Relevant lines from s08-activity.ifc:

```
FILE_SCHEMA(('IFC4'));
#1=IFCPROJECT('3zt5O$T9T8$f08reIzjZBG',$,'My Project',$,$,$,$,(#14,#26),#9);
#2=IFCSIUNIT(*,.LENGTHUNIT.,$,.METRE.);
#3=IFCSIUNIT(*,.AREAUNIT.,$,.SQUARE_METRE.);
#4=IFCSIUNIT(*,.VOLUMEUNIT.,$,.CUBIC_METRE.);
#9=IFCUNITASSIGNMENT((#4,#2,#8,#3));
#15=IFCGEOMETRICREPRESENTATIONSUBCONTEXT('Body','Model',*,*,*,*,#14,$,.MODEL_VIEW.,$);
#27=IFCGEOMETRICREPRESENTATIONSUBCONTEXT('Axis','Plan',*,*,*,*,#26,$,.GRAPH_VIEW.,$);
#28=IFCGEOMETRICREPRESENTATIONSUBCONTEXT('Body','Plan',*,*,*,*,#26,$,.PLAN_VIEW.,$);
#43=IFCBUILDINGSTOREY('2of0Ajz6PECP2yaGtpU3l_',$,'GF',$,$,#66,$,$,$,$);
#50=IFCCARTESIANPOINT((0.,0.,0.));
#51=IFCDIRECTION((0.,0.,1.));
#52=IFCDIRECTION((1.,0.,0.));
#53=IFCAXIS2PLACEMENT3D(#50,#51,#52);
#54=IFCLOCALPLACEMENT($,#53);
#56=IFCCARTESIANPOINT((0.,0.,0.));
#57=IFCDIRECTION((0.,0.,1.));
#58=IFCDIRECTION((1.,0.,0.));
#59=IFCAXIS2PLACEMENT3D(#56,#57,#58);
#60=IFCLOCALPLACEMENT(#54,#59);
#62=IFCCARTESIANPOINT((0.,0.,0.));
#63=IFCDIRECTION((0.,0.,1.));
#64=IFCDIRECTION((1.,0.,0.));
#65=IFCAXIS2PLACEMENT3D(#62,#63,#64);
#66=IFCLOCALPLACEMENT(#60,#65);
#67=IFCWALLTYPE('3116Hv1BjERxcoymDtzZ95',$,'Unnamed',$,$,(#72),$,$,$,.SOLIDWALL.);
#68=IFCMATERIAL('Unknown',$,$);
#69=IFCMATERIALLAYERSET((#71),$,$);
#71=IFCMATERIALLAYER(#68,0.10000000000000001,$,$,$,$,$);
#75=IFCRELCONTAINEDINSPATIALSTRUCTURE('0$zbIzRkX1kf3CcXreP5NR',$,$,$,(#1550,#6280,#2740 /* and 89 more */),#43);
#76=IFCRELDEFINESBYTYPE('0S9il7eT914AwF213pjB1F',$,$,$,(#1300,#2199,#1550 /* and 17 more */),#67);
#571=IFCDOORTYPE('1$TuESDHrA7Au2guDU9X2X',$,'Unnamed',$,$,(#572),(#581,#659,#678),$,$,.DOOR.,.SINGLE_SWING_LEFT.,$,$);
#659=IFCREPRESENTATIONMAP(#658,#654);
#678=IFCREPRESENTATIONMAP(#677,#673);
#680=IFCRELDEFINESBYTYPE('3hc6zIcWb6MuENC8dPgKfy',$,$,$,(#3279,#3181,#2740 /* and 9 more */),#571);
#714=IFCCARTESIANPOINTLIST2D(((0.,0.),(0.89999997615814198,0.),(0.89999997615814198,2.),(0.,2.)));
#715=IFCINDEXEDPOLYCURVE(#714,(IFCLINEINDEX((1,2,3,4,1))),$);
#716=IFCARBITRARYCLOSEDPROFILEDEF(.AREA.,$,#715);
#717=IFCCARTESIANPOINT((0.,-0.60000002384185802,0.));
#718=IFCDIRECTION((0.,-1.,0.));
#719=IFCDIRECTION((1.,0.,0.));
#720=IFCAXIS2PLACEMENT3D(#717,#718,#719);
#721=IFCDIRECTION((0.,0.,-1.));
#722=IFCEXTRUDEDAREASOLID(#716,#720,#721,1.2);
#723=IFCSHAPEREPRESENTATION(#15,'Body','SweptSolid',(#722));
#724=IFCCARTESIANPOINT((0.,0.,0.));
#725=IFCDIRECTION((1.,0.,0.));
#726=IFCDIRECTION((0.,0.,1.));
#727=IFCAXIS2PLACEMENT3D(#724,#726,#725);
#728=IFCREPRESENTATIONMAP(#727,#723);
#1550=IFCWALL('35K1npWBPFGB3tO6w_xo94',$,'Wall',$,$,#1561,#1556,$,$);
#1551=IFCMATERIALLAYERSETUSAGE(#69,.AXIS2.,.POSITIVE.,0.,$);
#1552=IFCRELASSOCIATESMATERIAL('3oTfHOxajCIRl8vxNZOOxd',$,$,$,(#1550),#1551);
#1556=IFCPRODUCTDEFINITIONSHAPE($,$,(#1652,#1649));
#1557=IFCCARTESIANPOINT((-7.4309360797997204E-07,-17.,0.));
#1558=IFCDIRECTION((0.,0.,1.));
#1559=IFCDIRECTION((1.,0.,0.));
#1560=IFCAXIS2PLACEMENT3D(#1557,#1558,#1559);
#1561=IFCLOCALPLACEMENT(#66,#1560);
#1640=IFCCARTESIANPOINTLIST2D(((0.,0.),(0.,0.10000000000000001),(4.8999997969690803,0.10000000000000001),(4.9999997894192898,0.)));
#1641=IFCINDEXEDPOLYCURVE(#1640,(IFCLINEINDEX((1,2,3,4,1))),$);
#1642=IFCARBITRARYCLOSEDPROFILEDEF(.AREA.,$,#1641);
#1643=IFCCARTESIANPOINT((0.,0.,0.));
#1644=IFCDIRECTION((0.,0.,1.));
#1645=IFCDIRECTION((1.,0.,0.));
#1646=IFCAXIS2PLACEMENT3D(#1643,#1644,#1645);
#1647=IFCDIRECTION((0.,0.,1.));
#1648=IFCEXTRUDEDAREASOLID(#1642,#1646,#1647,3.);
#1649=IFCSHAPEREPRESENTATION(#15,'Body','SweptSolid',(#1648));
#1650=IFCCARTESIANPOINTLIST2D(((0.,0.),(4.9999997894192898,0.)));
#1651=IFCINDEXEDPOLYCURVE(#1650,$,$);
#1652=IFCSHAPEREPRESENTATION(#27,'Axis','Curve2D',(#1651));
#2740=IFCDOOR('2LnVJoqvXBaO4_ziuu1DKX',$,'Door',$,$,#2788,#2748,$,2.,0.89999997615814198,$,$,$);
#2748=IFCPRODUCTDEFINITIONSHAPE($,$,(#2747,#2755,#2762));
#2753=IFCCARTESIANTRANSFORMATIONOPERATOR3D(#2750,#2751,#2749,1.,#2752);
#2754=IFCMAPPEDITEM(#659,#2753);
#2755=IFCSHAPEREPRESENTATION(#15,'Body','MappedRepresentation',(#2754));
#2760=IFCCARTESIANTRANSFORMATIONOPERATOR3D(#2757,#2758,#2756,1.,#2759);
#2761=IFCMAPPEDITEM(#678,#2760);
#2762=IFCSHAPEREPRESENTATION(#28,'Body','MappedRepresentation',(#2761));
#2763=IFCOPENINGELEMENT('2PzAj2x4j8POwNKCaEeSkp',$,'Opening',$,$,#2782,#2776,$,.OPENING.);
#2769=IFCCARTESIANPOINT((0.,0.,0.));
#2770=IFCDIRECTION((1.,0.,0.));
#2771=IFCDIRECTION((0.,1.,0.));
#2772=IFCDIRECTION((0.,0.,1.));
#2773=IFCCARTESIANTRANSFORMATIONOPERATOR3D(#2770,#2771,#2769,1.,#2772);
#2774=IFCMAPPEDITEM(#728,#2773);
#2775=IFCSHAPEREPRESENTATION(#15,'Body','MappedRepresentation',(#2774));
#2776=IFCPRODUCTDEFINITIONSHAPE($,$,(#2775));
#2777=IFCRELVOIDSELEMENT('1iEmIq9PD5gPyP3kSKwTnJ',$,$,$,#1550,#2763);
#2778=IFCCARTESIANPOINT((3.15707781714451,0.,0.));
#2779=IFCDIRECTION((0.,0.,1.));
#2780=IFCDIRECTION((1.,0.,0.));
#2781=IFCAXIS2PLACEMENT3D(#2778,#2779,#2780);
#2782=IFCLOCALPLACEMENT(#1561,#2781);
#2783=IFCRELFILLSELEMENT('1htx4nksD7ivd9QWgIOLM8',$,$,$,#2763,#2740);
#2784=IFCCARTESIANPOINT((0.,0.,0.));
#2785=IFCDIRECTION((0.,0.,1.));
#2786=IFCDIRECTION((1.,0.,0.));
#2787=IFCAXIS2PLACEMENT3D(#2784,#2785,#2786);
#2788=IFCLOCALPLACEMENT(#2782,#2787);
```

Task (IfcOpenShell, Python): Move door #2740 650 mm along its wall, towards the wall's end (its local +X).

```python
import ifcopenshell
import ifcopenshell.api.geometry
import ifcopenshell.util.placement
import ifcopenshell.util.unit

model = ifcopenshell.open("s08-activity.ifc")
unit_scale = ifcopenshell.util.unit.calculate_unit_scale(model)

door = model.by_id(2740)
opening = door.FillsVoids[0].RelatingOpeningElement
wall = opening.VoidsElements[0].RelatingBuildingElement

wall_matrix = ifcopenshell.util.placement.get_local_placement(wall.ObjectPlacement)
shift = wall_matrix[:3, 0] * 0.65 / unit_scale
before = ifcopenshell.util.placement.get_local_placement(door.ObjectPlacement)[:3, 3].copy()

# The door is placed relative to its opening, so it follows when the opening moves.
matrix = ifcopenshell.util.placement.get_local_placement(opening.ObjectPlacement)
matrix[:3, 3] += shift
ifcopenshell.api.geometry.edit_object_placement(
    model, product=opening, matrix=matrix, is_si=False, should_transform_children=True
)

after = ifcopenshell.util.placement.get_local_placement(door.ObjectPlacement)[:3, 3]
print("door moved by", (after - before).round(3) + 0.0)

model.write("s08-activity-out.ifc")
```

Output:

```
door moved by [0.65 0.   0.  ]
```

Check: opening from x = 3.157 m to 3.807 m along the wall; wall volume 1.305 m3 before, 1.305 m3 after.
